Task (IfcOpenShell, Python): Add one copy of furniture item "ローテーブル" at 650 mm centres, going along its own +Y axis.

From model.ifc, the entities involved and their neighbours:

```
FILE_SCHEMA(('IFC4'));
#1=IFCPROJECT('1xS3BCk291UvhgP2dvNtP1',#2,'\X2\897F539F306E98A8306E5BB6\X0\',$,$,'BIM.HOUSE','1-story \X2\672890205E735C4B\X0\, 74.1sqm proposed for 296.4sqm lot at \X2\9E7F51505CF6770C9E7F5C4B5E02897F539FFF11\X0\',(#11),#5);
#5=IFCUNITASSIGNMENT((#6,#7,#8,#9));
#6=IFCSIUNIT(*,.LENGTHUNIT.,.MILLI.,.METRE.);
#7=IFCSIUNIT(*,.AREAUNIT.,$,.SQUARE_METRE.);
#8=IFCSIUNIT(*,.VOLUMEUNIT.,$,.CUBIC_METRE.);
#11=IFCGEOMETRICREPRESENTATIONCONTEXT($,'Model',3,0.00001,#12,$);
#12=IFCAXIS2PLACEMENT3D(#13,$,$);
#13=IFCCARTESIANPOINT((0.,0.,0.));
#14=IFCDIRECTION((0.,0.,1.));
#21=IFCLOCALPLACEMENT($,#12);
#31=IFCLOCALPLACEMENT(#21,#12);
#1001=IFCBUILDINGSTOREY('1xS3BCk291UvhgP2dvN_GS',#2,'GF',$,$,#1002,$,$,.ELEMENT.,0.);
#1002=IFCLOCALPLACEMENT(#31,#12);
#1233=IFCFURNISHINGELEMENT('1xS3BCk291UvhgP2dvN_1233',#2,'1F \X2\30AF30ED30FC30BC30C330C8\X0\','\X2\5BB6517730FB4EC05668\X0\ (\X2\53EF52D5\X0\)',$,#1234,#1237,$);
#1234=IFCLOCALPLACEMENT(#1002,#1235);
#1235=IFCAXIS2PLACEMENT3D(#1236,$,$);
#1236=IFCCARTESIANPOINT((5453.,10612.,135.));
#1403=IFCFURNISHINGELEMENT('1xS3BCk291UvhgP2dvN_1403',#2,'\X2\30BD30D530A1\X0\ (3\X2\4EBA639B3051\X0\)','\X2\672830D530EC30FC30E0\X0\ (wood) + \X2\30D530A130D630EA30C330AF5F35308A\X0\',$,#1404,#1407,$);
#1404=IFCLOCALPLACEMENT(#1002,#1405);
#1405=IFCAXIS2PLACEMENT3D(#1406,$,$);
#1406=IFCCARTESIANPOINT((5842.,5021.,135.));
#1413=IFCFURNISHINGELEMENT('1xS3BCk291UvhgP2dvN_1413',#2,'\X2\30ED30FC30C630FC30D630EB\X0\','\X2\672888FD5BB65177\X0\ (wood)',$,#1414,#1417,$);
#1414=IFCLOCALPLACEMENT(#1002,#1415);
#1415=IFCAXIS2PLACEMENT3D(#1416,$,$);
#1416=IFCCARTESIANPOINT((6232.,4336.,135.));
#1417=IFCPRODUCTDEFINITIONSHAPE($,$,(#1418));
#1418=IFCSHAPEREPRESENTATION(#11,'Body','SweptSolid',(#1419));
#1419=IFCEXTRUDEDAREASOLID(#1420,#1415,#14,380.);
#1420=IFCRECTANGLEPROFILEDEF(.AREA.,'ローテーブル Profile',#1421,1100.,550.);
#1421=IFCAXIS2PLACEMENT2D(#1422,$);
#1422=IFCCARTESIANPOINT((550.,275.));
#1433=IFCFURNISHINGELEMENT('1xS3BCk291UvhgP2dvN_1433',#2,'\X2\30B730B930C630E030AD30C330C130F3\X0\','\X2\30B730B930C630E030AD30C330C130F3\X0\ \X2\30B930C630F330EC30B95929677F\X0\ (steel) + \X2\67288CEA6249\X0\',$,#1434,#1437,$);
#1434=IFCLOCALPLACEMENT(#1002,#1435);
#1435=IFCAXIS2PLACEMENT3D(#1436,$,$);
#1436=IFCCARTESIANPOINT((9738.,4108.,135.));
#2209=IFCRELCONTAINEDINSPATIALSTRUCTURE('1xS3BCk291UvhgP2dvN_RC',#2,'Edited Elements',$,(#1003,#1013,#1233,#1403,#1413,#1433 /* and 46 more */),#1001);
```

```python
import ifcopenshell
import ifcopenshell.api.geometry
import ifcopenshell.api.root
import ifcopenshell.util.element
import ifcopenshell.util.placement

model = ifcopenshell.open("model.ifc")


def reuse_history(source, copy):
    """copy_class also copies each property set's owner history, people and application; keep the originals."""
    for rel in copy.IsDefinedBy:
        if rel.is_a("IfcRelDefinesByProperties") and (history := rel.RelatingPropertyDefinition.OwnerHistory):
            rel.RelatingPropertyDefinition.OwnerHistory = source.OwnerHistory
            ifcopenshell.util.element.remove_deep2(model, history)


source = model.by_guid("1xS3BCk291UvhgP2dvN_1413")
base = ifcopenshell.util.placement.get_local_placement(source.ObjectPlacement)
step = base[:3, 1] * 650.0

for i in range(1, 2):
    copy = ifcopenshell.api.root.copy_class(model, product=source)
    copy.Representation = ifcopenshell.util.element.copy_deep(
        model, source.Representation, exclude=["IfcGeometricRepresentationContext", "IfcRepresentationMap"]
    )
    reuse_history(source, copy)
    matrix = base.copy()
    matrix[:3, 3] += i * step
    print("added at", matrix[:3, 3].round(3) + 0.0)
    ifcopenshell.api.geometry.edit_object_placement(model, product=copy, matrix=matrix, is_si=False)

model.write("model_edited.ifc")
```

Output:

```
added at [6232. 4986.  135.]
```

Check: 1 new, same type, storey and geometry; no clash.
